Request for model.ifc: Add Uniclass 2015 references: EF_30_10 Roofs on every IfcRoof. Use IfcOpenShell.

First a look at what the model holds.

```python
import ifcopenshell

model = ifcopenshell.open("model.ifc")
print(model.schema)
print("classifications:", [c.Name for c in model.by_type("IfcClassification")])
for ifc_class in ("IfcDoor", "IfcRoof", "IfcStair", "IfcWall", "IfcWindow"):
    print(ifc_class, len(model.by_type(ifc_class)))
```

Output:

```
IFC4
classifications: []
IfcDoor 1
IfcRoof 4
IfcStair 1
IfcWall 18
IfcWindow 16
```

```python
import ifcopenshell
import ifcopenshell.api.classification

model = ifcopenshell.open("model.ifc")

system = ifcopenshell.api.classification.add_classification(model, classification="Uniclass 2015")

codes = {
    "IfcRoof": ("EF_30_10", "Roofs"),
}
for ifc_class, (code, name) in codes.items():
    products = model.by_type(ifc_class)
    ifcopenshell.api.classification.add_reference(
        model, products=products, classification=system, identification=code, name=name
    )
    print(code, len(products))

model.write("model_updated.ifc")
```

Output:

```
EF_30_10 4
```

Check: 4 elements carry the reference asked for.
